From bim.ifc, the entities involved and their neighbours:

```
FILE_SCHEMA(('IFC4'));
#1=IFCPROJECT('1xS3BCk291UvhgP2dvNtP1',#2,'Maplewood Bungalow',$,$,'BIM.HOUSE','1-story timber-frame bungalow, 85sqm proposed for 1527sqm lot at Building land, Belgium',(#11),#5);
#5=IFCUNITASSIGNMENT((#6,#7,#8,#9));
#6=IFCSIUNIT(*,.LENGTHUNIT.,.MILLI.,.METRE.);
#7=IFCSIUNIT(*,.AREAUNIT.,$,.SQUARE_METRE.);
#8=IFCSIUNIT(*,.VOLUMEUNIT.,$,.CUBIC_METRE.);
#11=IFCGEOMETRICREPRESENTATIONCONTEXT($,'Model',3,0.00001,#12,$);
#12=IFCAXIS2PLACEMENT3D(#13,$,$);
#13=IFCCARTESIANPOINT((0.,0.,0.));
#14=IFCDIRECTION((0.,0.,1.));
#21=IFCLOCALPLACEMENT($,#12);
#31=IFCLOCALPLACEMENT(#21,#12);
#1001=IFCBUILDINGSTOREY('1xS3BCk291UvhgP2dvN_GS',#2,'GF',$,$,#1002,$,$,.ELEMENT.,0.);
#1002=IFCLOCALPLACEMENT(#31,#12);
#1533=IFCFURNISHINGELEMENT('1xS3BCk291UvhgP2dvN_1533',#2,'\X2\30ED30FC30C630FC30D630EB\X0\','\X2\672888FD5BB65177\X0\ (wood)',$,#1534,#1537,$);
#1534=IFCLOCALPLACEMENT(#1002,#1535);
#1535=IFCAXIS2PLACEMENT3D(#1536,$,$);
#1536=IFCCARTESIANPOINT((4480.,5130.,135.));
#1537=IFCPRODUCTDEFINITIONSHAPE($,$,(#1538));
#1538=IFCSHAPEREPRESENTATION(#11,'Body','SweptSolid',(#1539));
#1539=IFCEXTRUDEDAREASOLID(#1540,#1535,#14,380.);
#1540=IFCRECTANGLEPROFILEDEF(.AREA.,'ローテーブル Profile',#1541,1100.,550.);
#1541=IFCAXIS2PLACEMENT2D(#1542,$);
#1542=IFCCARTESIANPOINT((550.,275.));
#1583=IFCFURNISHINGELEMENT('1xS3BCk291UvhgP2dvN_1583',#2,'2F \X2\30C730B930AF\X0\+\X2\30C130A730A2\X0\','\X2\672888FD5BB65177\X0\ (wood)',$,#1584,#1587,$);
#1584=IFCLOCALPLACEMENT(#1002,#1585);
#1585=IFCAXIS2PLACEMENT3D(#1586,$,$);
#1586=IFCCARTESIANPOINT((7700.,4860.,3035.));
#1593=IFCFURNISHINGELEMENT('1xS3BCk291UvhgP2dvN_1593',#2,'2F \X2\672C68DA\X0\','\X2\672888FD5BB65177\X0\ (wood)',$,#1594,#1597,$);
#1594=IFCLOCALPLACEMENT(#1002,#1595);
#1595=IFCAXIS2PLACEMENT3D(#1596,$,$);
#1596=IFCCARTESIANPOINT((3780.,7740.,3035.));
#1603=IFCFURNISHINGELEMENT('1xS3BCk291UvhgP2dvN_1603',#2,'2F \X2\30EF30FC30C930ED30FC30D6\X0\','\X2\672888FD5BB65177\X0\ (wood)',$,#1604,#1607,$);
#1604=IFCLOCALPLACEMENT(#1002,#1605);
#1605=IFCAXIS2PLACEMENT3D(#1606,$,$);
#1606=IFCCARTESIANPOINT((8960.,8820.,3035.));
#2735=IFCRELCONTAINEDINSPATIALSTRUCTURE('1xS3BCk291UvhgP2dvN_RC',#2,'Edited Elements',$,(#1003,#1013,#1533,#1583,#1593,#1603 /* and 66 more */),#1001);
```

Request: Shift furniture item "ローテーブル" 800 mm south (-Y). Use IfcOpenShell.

```python
import ifcopenshell
import ifcopenshell.api.geometry
import ifcopenshell.util.placement

model = ifcopenshell.open("bim.ifc")

item = model.by_guid("1xS3BCk291UvhgP2dvN_1533")
matrix = ifcopenshell.util.placement.get_local_placement(item.ObjectPlacement)
matrix[1, 3] -= 800.0
ifcopenshell.api.geometry.edit_object_placement(model, product=item, matrix=matrix, is_si=False)

print(ifcopenshell.util.placement.get_local_placement(item.ObjectPlacement).round(3) + 0.0)

model.write("bim-out.ifc")
```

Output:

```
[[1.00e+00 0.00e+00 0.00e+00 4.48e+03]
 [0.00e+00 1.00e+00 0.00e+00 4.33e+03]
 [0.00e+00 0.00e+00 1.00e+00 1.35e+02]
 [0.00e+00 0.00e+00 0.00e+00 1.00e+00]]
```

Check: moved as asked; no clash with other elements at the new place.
